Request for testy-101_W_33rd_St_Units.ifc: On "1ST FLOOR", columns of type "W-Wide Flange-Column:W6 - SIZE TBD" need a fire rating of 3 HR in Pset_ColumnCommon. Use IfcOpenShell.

First a look at what the model holds.

```python
import ifcopenshell
import ifcopenshell.util.element

model = ifcopenshell.open("testy-101_W_33rd_St_Units.ifc")
print(model.schema)
storey = next(s for s in model.by_type("IfcBuildingStorey") if s.Name == "1ST FLOOR")
columns = [e for e in ifcopenshell.util.element.get_decomposition(storey) if e.is_a("IfcColumn")]
seen = {}
for e in columns:
    element_type = ifcopenshell.util.element.get_type(e)
    key = (element_type.Name if element_type != e and element_type else None, ifcopenshell.util.element.get_pset(e, "Pset_ColumnCommon", "FireRating"))
    seen[key] = seen.get(key, 0) + 1
for (name, value), count in sorted(seen.items(), key=str):
    print(count, "x", name, "|", value)
```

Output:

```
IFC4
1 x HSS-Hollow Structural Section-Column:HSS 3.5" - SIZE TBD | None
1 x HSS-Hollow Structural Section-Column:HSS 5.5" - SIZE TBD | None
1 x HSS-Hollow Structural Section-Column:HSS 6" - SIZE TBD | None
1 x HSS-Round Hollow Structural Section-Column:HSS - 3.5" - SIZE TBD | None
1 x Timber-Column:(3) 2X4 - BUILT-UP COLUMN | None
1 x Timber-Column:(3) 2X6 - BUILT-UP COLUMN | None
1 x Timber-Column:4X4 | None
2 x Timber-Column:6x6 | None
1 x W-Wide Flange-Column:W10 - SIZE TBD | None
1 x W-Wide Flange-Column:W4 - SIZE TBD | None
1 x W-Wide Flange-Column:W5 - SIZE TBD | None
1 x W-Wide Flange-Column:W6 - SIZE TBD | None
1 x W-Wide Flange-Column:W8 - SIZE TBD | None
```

```python
import ifcopenshell
import ifcopenshell.api.pset
import ifcopenshell.util.element

model = ifcopenshell.open("testy-101_W_33rd_St_Units.ifc")

storey = next(s for s in model.by_type("IfcBuildingStorey") if s.Name == "1ST FLOOR")
columns = [e for e in ifcopenshell.util.element.get_decomposition(storey) if e.is_a("IfcColumn")]

count = 0
for e in columns:
    element_type = ifcopenshell.util.element.get_type(e)
    if element_type in (None, e) or element_type.Name != "W-Wide Flange-Column:W6 - SIZE TBD":
        continue
    # add_pset returns the element's existing set when there is one.
    pset = ifcopenshell.api.pset.add_pset(model, product=e, name="Pset_ColumnCommon")
    ifcopenshell.api.pset.edit_pset(model, pset=pset, properties={"FireRating": "3 HR"})
    count += 1

print(count, "columns updated")

model.write("testy-101_W_33rd_St_Units_rev.ifc")
```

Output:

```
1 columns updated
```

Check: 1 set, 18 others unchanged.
